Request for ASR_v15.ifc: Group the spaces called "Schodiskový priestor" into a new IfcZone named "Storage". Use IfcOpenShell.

First a look at what the model holds.

```python
import ifcopenshell

model = ifcopenshell.open("ASR_v15.ifc")
print(model.schema)
seen = {}
for space in model.by_type("IfcSpace"):
    seen[space.LongName] = seen.get(space.LongName, 0) + 1
for name, count in sorted(seen.items(), key=str):
    print(count, "x", name)
print("zones:", [z.Name for z in model.by_type("IfcZone")][:20])
```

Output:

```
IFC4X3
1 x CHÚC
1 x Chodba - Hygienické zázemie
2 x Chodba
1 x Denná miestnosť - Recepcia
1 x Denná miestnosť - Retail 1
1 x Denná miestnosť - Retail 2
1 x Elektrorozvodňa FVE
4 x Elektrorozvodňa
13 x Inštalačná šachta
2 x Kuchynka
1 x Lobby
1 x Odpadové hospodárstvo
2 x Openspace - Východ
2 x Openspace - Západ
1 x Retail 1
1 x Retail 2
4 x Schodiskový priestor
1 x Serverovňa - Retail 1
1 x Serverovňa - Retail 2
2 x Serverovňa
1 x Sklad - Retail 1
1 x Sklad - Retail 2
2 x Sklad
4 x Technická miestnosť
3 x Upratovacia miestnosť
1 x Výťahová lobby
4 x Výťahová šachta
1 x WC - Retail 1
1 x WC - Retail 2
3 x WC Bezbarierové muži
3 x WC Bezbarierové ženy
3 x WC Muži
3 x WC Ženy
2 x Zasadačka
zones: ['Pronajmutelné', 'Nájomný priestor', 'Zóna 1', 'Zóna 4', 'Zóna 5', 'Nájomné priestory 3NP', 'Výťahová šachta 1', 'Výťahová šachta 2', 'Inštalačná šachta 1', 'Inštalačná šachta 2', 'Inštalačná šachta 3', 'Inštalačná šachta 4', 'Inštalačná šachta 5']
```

```python
import ifcopenshell
import ifcopenshell.api.group
import ifcopenshell.api.root

model = ifcopenshell.open("ASR_v15.ifc")

names = {"Schodiskový priestor"}
spaces = [s for s in model.by_type("IfcSpace") if s.LongName in names]

zone = ifcopenshell.api.root.create_entity(model, ifc_class="IfcZone", name="Storage")
ifcopenshell.api.group.assign_group(model, products=spaces, group=zone)
print(len(spaces), "spaces in", zone.Name)

model.write("ASR_v15_rev.ifc")
```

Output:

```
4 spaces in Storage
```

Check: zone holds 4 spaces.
